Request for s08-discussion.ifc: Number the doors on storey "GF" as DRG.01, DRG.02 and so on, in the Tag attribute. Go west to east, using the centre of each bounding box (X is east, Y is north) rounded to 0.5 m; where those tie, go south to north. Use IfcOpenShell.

First a look at what the model holds.

```python
import ifcopenshell
import ifcopenshell.util.element
import ifcopenshell.util.placement

model = ifcopenshell.open("s08-discussion.ifc")
print(model.schema)
storey = next(s for s in model.by_type("IfcBuildingStorey") if s.Name == "GF")
doors = [e for e in ifcopenshell.util.element.get_decomposition(storey) if e.is_a("IfcDoor")]
for e in sorted(doors, key=lambda e: e.id()):
    origin = ifcopenshell.util.placement.get_local_placement(e.ObjectPlacement)[:3, 3]
    print(e.id(), e.Tag, e.Name, origin.round(2) + 0.0, sep=" | ")
```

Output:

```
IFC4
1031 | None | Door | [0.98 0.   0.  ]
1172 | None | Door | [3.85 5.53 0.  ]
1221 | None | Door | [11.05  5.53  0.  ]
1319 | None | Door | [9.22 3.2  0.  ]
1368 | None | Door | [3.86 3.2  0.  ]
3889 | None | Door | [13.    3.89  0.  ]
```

```python
import ifcopenshell
import ifcopenshell.geom
import ifcopenshell.util.element
import ifcopenshell.util.shape

model = ifcopenshell.open("s08-discussion.ifc")
settings = ifcopenshell.geom.settings()
settings.set("use-world-coords", True)


def centre(element):
    shape = ifcopenshell.geom.create_shape(settings, element)
    return ifcopenshell.util.shape.get_bbox_centroid(shape.geometry)


storey = next(s for s in model.by_type("IfcBuildingStorey") if s.Name == "GF")
doors = [e for e in ifcopenshell.util.element.get_decomposition(storey) if e.is_a("IfcDoor")]

# Insertion points can sit at a corner or the storey origin, so sort by the geometry (in metres).
centres = {e: centre(e) for e in doors}
doors.sort(key=lambda e: (round(centres[e][0] / 0.5), centres[e][1]))

for i, e in enumerate(doors, start=1):
    number = f"DRG.{i:02d}"
    e.Tag = number
    print(e.id(), number)

model.write("s08-discussion_rev.ifc")
```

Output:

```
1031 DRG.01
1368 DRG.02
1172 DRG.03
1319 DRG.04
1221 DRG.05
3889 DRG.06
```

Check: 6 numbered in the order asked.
